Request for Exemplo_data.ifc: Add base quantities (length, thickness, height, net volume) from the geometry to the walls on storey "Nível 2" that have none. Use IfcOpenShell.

First a look at what the model holds.

```python
import ifcopenshell
import ifcopenshell.util.element
import ifcopenshell.util.unit

model = ifcopenshell.open("Exemplo_data.ifc")
print(model.schema)
for unit_type in ("LENGTHUNIT", "AREAUNIT", "VOLUMEUNIT"):
    print(unit_type, ifcopenshell.util.unit.calculate_unit_scale(model, unit_type))
storey = next(s for s in model.by_type("IfcBuildingStorey") if s.Name == "Nível 2")
walls = [e for e in ifcopenshell.util.element.get_decomposition(storey) if e.is_a("IfcWall")]
for e in sorted(walls, key=lambda e: e.id()):
    print(e.id(), e.is_a(), e.Name, list(ifcopenshell.util.element.get_psets(e, qtos_only=True)), sep=" | ")
```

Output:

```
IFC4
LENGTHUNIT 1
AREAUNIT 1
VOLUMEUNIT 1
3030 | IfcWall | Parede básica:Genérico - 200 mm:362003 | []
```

```python
import ifcopenshell
import ifcopenshell.api.pset
import ifcopenshell.geom
import ifcopenshell.util.element
import ifcopenshell.util.shape
import ifcopenshell.util.unit

model = ifcopenshell.open("Exemplo_data.ifc")
unit_scale = ifcopenshell.util.unit.calculate_unit_scale(model)
volume_scale = ifcopenshell.util.unit.calculate_unit_scale(model, "VOLUMEUNIT")
settings = ifcopenshell.geom.settings()

storey = next(s for s in model.by_type("IfcBuildingStorey") if s.Name == "Nível 2")
walls = [e for e in ifcopenshell.util.element.get_decomposition(storey) if e.is_a("IfcWall")]

for e in sorted(walls, key=lambda e: e.id()):
    if ifcopenshell.util.element.get_psets(e, qtos_only=True, should_inherit=False):
        continue
    # Geometry comes back in metres, in the element's own axes.
    shape = ifcopenshell.geom.create_shape(settings, e)
    values = {
        "Length": ifcopenshell.util.shape.get_x(shape.geometry) / unit_scale,
        "Width": ifcopenshell.util.shape.get_y(shape.geometry) / unit_scale,
        "Height": ifcopenshell.util.shape.get_z(shape.geometry) / unit_scale,
        "NetVolume": ifcopenshell.util.shape.get_volume(shape.geometry) / volume_scale,
    }
    qto = ifcopenshell.api.pset.add_qto(model, product=e, name="Qto_WallBaseQuantities")
    ifcopenshell.api.pset.edit_qto(model, qto=qto, properties=values)
    print(e.id(), {k: round(v, 3) for k, v in values.items()})

model.write("Exemplo_data_v2.ifc")
```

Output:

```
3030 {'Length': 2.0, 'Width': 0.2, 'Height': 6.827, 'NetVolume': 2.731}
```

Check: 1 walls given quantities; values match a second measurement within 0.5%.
